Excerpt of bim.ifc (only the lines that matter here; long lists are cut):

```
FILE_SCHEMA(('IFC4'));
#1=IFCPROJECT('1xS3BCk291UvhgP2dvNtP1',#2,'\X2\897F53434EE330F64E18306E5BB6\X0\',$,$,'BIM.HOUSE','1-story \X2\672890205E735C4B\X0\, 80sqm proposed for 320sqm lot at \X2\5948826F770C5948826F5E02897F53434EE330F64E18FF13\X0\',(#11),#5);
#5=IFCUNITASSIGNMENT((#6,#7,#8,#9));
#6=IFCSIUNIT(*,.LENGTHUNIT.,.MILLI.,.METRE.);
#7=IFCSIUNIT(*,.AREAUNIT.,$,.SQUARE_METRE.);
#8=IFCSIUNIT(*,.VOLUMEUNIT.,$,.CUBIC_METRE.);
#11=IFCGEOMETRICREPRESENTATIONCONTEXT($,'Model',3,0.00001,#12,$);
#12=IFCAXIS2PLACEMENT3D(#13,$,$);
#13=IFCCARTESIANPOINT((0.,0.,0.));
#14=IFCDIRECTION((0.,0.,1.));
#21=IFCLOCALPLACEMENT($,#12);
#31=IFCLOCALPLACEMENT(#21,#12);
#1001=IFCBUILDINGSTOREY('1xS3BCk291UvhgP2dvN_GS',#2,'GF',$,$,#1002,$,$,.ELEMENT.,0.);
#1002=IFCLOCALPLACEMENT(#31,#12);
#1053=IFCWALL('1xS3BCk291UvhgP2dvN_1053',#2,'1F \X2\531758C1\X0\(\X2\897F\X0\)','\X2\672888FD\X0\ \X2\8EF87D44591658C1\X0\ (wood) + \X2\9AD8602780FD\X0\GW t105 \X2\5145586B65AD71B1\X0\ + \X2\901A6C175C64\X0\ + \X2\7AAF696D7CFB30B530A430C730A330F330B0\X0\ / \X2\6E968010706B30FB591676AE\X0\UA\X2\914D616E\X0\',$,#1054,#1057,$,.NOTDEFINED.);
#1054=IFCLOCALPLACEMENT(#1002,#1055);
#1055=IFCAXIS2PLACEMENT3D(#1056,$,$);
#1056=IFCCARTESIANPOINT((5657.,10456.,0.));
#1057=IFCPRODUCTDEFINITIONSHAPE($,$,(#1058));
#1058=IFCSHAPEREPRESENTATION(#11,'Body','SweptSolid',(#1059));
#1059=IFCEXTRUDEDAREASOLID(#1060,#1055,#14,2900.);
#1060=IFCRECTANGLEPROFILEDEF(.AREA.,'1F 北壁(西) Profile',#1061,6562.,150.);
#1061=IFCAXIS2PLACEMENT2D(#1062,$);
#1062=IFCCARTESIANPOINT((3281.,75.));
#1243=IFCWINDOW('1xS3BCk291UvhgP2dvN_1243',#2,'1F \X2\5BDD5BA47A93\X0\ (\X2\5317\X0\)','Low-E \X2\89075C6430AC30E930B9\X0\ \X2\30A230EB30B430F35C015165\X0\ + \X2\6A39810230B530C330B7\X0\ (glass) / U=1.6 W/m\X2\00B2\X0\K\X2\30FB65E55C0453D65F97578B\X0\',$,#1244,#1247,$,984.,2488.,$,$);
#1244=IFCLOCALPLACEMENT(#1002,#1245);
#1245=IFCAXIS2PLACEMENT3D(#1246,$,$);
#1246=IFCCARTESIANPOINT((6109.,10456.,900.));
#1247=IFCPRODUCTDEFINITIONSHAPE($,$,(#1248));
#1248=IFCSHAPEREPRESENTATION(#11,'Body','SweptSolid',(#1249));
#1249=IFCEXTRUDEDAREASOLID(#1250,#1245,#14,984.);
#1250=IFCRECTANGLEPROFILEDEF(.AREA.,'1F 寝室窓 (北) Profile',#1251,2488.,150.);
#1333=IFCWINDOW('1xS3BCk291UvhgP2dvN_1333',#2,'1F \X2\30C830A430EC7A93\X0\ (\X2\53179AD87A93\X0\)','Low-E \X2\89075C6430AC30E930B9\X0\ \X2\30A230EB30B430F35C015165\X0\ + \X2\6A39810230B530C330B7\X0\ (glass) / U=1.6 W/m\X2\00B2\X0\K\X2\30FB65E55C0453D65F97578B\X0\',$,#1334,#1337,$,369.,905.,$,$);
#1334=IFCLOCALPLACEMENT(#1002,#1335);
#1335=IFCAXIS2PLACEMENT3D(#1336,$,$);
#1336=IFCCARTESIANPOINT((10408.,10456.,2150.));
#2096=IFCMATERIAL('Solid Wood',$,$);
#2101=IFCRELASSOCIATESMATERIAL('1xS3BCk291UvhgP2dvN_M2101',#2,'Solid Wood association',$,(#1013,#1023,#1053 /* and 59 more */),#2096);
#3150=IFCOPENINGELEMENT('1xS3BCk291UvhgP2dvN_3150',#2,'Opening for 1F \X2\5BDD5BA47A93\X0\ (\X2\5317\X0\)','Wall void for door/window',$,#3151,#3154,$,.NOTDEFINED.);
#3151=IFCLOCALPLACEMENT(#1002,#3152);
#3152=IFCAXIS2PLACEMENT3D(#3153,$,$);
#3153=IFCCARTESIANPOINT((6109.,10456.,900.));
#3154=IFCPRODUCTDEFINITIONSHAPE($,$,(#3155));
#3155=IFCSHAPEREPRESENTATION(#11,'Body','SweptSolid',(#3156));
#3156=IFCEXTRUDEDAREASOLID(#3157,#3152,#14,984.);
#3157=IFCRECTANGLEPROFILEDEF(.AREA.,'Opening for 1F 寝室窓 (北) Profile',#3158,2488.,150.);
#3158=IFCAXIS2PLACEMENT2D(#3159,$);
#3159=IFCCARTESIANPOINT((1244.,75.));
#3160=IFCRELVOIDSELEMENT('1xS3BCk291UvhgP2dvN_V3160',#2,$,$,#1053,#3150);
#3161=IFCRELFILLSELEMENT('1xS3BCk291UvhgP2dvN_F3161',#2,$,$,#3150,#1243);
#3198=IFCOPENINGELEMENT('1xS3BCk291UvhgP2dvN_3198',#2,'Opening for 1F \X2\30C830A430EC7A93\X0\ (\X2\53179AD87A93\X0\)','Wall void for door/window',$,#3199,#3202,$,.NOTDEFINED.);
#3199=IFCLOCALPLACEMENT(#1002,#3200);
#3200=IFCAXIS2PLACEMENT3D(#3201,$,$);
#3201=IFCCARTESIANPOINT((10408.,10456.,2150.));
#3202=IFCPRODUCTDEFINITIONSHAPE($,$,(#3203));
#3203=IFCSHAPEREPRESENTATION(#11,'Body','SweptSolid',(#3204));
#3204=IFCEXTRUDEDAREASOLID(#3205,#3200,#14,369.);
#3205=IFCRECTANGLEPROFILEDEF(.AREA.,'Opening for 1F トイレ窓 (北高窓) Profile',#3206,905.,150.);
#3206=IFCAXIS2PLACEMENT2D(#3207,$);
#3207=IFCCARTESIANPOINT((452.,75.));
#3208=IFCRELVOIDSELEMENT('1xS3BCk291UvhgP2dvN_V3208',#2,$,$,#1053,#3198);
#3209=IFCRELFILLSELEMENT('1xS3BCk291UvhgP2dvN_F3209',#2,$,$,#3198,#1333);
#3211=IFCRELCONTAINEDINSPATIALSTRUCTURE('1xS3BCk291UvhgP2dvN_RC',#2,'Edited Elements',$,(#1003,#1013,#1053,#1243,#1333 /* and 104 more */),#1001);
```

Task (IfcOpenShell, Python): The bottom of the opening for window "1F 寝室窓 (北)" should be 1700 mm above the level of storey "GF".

```python
import numpy as np
import ifcopenshell
import ifcopenshell.api.geometry
import ifcopenshell.geom
import ifcopenshell.util.element
import ifcopenshell.util.placement
import ifcopenshell.util.shape
import ifcopenshell.util.unit

model = ifcopenshell.open("bim.ifc")
unit_scale = ifcopenshell.util.unit.calculate_unit_scale(model)

window = model.by_guid("1xS3BCk291UvhgP2dvN_1243")
opening = window.FillsVoids[0].RelatingOpeningElement
storey = ifcopenshell.util.element.get_container(window, ifc_class="IfcBuildingStorey")
level = ifcopenshell.util.placement.get_local_placement(storey.ObjectPlacement)[2, 3]

# The opening's origin need not be at the sill, so measure its lowest point.
shape = ifcopenshell.geom.create_shape(ifcopenshell.geom.settings(), opening)
bottom = ifcopenshell.util.shape.get_shape_bottom_elevation(shape, shape.geometry) / unit_scale
dz = level + 1.7 / unit_scale - bottom

shift = np.array([0.0, 0.0, dz])
# The window is not placed relative to its opening, so move both.
for product in (opening, window):
    matrix = ifcopenshell.util.placement.get_local_placement(product.ObjectPlacement)
    matrix[:3, 3] += shift
    ifcopenshell.api.geometry.edit_object_placement(model, product=product, matrix=matrix, is_si=False)

print(f"moved by {dz * unit_scale:+.3f} m")

model.write("bim_updated.ifc")
```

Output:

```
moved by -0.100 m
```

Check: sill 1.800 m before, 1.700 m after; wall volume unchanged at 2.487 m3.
